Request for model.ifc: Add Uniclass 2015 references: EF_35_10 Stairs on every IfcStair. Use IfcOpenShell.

First a look at what the model holds.

```python
import ifcopenshell

model = ifcopenshell.open("model.ifc")
print(model.schema)
print("classifications:", [c.Name for c in model.by_type("IfcClassification")])
for ifc_class in ("IfcDoor", "IfcRoof", "IfcStair", "IfcWall", "IfcWindow"):
    print(ifc_class, len(model.by_type(ifc_class)))
```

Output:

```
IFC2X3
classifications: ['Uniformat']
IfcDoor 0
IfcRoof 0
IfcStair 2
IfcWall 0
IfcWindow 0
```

```python
import ifcopenshell
import ifcopenshell.api.classification

model = ifcopenshell.open("model.ifc")

# IFC2X3 requires Source and Edition and has no link from the project to the system.
system = model.create_entity("IfcClassification", Source="NBS", Edition="2015", Name="Uniclass 2015")

codes = {
    "IfcStair": ("EF_35_10", "Stairs"),
}
for ifc_class, (code, name) in codes.items():
    products = model.by_type(ifc_class)
    ifcopenshell.api.classification.add_reference(
        model, products=products, classification=system, identification=code, name=name
    )
    print(code, len(products))

model.write("model_edited.ifc")
```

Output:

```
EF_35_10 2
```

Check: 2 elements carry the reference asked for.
